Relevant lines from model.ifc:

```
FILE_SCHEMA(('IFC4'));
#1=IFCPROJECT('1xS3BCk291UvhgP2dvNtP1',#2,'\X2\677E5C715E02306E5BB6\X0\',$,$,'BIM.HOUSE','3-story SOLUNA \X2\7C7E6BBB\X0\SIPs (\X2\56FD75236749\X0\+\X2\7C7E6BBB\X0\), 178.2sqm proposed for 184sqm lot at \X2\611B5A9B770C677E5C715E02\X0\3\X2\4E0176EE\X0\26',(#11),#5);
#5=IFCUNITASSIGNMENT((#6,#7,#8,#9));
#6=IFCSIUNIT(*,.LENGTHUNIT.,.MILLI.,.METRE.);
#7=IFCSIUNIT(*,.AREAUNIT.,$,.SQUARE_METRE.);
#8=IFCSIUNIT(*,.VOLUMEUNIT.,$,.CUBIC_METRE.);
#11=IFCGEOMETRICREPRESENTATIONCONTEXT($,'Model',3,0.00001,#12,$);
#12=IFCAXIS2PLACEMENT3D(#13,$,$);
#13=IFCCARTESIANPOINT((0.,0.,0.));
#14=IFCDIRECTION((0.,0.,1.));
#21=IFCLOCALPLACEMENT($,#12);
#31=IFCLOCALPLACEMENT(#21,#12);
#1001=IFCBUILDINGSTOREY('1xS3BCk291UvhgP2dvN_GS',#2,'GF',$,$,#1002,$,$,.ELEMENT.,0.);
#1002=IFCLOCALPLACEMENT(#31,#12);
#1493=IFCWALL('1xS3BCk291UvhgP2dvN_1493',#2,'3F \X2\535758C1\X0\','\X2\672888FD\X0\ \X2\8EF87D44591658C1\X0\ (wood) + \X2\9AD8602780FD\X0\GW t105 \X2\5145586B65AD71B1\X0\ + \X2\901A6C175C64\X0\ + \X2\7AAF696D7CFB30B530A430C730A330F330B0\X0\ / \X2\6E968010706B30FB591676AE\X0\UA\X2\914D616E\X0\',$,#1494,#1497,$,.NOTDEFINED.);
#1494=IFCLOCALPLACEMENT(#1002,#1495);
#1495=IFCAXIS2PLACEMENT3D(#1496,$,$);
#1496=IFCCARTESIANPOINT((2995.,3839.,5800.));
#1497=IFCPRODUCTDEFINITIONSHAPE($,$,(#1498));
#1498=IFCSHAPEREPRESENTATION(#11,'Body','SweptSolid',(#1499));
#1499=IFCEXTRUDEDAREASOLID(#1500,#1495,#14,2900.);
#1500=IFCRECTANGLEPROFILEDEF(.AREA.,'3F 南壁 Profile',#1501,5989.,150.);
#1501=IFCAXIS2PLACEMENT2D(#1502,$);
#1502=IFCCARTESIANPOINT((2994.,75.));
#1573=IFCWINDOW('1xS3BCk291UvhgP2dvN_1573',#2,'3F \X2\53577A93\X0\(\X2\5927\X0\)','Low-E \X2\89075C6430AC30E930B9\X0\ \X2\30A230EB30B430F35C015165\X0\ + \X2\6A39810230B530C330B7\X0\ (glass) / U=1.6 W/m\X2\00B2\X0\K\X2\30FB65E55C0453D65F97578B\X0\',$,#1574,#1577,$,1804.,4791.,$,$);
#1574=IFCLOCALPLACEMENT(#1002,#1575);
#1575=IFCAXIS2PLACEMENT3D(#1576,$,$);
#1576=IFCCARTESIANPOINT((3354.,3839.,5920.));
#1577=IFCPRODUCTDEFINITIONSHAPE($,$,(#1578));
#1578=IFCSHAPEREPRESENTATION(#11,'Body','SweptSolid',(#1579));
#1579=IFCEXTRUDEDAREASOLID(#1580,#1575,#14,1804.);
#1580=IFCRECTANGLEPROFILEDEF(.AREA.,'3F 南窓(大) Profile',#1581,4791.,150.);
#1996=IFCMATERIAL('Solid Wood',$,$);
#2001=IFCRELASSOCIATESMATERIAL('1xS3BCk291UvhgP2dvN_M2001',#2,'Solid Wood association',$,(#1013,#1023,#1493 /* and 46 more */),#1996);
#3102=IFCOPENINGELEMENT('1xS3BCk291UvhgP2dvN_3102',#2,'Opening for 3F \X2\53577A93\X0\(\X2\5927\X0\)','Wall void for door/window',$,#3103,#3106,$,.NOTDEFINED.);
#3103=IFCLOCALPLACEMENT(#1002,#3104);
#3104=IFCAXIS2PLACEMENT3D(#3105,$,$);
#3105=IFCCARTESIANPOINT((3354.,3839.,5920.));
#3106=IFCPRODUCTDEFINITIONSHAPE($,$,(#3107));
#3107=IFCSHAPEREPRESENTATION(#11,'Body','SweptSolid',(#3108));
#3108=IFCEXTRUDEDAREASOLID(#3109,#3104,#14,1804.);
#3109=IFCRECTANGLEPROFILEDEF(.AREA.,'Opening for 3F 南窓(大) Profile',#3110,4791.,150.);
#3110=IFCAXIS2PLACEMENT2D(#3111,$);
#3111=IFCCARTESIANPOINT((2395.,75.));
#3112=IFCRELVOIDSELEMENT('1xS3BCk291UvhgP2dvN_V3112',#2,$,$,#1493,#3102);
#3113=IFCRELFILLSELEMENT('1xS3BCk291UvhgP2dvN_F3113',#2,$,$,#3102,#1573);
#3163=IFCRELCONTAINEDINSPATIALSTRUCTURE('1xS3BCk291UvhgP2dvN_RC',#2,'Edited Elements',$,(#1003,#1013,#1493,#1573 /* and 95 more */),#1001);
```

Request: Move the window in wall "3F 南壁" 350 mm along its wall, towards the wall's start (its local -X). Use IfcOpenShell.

```python
import ifcopenshell
import ifcopenshell.api.geometry
import ifcopenshell.util.placement
import ifcopenshell.util.unit

model = ifcopenshell.open("model.ifc")
unit_scale = ifcopenshell.util.unit.calculate_unit_scale(model)

window = model.by_guid("1xS3BCk291UvhgP2dvN_1573")
opening = window.FillsVoids[0].RelatingOpeningElement
wall = opening.VoidsElements[0].RelatingBuildingElement

wall_matrix = ifcopenshell.util.placement.get_local_placement(wall.ObjectPlacement)
shift = wall_matrix[:3, 0] * -0.35 / unit_scale
before = ifcopenshell.util.placement.get_local_placement(window.ObjectPlacement)[:3, 3].copy()

# The window is not placed relative to its opening, so move both.
for product in (opening, window):
    matrix = ifcopenshell.util.placement.get_local_placement(product.ObjectPlacement)
    matrix[:3, 3] += shift
    ifcopenshell.api.geometry.edit_object_placement(model, product=product, matrix=matrix, is_si=False)

after = ifcopenshell.util.placement.get_local_placement(window.ObjectPlacement)[:3, 3]
print("window moved by", (after - before).round(3) + 0.0)

model.write("model_updated.ifc")
```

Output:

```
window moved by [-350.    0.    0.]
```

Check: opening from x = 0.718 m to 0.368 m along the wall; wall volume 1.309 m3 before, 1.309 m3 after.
